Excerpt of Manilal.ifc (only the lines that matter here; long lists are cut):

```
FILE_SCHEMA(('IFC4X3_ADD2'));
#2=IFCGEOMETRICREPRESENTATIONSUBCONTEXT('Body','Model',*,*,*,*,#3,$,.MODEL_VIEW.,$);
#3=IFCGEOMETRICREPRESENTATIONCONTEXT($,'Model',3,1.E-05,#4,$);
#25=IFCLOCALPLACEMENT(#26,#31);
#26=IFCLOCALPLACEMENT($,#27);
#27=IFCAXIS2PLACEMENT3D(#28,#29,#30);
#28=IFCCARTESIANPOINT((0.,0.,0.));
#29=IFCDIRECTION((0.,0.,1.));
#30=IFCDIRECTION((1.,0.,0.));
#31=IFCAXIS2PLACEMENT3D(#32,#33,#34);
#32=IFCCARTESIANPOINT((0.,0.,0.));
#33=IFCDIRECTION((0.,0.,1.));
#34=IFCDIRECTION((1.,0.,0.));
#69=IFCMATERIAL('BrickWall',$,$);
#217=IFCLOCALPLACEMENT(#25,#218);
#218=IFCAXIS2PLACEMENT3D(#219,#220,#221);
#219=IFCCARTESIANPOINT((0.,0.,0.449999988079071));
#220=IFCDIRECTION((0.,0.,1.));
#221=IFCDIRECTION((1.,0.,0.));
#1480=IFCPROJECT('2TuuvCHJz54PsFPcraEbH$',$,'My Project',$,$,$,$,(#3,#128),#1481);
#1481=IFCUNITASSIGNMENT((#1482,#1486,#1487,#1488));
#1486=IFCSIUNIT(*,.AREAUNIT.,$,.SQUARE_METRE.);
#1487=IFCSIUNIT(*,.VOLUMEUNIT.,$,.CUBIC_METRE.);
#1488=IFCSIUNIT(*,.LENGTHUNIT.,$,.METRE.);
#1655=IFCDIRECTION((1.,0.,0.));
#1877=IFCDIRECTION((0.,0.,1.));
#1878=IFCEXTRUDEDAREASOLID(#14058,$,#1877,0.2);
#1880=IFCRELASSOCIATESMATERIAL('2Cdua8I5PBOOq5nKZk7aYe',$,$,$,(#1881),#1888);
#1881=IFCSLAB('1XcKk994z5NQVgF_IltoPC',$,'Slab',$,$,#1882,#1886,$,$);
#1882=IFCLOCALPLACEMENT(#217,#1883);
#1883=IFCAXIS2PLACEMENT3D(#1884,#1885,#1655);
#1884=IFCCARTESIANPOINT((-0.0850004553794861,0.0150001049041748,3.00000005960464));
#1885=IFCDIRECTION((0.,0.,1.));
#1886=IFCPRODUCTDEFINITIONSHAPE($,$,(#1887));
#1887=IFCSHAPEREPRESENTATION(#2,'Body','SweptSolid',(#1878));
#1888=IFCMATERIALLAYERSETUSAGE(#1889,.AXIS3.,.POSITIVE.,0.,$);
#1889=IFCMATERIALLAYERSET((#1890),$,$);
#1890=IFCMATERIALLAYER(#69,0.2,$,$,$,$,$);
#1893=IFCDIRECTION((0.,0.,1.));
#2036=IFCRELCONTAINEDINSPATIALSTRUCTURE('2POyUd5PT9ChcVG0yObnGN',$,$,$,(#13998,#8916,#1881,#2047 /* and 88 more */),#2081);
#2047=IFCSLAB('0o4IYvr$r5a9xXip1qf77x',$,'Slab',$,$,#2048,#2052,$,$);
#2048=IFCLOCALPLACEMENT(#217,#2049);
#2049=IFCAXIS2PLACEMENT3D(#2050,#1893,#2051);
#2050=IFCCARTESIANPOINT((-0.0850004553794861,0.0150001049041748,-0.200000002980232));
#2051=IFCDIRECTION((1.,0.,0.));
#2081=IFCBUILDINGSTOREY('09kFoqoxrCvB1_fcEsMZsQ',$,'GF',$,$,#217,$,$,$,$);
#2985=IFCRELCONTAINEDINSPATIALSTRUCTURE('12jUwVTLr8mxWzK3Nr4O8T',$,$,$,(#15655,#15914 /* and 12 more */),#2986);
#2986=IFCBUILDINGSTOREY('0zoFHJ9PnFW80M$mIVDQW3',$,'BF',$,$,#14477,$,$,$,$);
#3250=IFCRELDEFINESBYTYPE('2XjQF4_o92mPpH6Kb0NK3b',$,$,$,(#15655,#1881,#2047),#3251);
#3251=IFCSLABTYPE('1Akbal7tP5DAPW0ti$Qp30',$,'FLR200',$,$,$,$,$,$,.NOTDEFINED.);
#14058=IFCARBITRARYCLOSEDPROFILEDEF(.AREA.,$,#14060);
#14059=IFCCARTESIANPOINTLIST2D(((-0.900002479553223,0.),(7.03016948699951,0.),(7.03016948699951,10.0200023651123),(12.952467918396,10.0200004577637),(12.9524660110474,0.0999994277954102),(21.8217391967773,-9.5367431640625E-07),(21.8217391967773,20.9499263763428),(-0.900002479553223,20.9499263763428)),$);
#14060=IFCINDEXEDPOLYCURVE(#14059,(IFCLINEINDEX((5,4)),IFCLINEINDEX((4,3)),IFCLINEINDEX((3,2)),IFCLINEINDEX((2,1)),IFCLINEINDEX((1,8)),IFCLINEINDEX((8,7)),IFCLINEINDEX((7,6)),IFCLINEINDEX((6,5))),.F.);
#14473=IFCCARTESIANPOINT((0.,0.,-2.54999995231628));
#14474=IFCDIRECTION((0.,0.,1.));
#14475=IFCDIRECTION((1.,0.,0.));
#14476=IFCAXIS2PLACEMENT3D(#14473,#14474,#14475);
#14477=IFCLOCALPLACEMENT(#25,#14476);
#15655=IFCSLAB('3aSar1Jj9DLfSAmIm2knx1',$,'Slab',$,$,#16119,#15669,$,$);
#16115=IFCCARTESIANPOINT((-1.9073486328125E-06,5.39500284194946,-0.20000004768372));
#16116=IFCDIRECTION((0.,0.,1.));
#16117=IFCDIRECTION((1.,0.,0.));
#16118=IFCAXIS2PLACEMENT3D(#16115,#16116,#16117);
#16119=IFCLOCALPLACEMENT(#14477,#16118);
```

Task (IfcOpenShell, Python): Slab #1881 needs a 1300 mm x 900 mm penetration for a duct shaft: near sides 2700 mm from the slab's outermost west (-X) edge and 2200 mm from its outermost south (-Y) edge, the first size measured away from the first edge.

```python
import numpy as np
import ifcopenshell
import ifcopenshell.api.feature
import ifcopenshell.api.geometry
import ifcopenshell.api.root
import ifcopenshell.geom
import ifcopenshell.util.placement
import ifcopenshell.util.representation
import ifcopenshell.util.shape
import ifcopenshell.util.unit

model = ifcopenshell.open("Manilal.ifc")
unit_scale = ifcopenshell.util.unit.calculate_unit_scale(model)
settings = ifcopenshell.geom.settings()


def volume(element):
    """Net volume in cubic metres, openings subtracted."""
    shape = ifcopenshell.geom.create_shape(settings, element)
    return ifcopenshell.util.shape.get_volume(shape.geometry)


slab = model.by_guid("1XcKk994z5NQVgF_IltoPC")
before = volume(slab)

# Extent in the slab's own axes, in metres. The edges named are its -X and -Y sides.
slab_shape = ifcopenshell.geom.create_shape(settings, slab)
vertices = ifcopenshell.util.shape.get_vertices(slab_shape.geometry)
x_min, y_min, bottom = vertices.min(axis=0)
top = vertices[:, 2].max()

opening = ifcopenshell.api.root.create_entity(model, ifc_class="IfcOpeningElement", name="Duct shaft opening", predefined_type="OPENING")
context = ifcopenshell.util.representation.get_context(model, "Model", "Body", "MODEL_VIEW")
width, depth = 1.3, 0.9
outline = [(0.0, 0.0), (width, 0.0), (width, depth), (0.0, depth), (0.0, 0.0)]
# Overshoot both faces by 50 mm so the cut is clean.
shape = ifcopenshell.api.geometry.add_slab_representation(
    model, context=context, depth=top - bottom + 0.1, polyline=outline
)
ifcopenshell.api.geometry.assign_representation(model, product=opening, representation=shape)

matrix = ifcopenshell.util.placement.get_local_placement(slab.ObjectPlacement)
matrix[:, 3] = matrix @ np.append(np.array([x_min + 2.7, y_min + 2.2, bottom - 0.05]) / unit_scale, 1.0)
ifcopenshell.api.geometry.edit_object_placement(model, product=opening, matrix=matrix, is_si=False)
ifcopenshell.api.feature.add_feature(model, feature=opening, element=slab)

after = volume(slab)

print(f"slab volume {before:.3f} -> {after:.3f} m3")

model.write("Manilal_updated.ifc")
```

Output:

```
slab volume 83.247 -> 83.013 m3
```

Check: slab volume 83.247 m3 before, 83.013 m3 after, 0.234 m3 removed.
